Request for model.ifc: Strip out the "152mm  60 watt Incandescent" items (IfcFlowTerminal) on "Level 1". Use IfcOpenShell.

First a look at what the model holds.

```python
import ifcopenshell
import ifcopenshell.util.element

model = ifcopenshell.open("model.ifc")
print(model.schema)
storey = next(s for s in model.by_type("IfcBuildingStorey") if s.Name == "Level 1")
terminals = [e for e in ifcopenshell.util.element.get_decomposition(storey) if e.is_a("IfcFlowTerminal")]
seen = {}
for e in terminals:
    element_type = ifcopenshell.util.element.get_type(e)
    name = element_type.Name if element_type not in (None, e) else None
    seen[name] = seen.get(name, 0) + 1
for name, count in sorted(seen.items(), key=str):
    print(count, "x", name)
```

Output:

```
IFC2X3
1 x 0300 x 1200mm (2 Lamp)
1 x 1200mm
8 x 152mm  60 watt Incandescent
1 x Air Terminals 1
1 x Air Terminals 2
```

```python
import ifcopenshell
import ifcopenshell.api.root
import ifcopenshell.util.element

model = ifcopenshell.open("model.ifc")

storey = next(s for s in model.by_type("IfcBuildingStorey") if s.Name == "Level 1")
terminals = [e for e in ifcopenshell.util.element.get_decomposition(storey) if e.is_a("IfcFlowTerminal")]
targets = [e for e in terminals if (t := ifcopenshell.util.element.get_type(e)) not in (None, e) and t.Name == "152mm  60 watt Incandescent"]

for e in targets:
    ifcopenshell.api.root.remove_product(model, product=e)
print(len(targets), "removed")

model.write("model_edited.ifc")
```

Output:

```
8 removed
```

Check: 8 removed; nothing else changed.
